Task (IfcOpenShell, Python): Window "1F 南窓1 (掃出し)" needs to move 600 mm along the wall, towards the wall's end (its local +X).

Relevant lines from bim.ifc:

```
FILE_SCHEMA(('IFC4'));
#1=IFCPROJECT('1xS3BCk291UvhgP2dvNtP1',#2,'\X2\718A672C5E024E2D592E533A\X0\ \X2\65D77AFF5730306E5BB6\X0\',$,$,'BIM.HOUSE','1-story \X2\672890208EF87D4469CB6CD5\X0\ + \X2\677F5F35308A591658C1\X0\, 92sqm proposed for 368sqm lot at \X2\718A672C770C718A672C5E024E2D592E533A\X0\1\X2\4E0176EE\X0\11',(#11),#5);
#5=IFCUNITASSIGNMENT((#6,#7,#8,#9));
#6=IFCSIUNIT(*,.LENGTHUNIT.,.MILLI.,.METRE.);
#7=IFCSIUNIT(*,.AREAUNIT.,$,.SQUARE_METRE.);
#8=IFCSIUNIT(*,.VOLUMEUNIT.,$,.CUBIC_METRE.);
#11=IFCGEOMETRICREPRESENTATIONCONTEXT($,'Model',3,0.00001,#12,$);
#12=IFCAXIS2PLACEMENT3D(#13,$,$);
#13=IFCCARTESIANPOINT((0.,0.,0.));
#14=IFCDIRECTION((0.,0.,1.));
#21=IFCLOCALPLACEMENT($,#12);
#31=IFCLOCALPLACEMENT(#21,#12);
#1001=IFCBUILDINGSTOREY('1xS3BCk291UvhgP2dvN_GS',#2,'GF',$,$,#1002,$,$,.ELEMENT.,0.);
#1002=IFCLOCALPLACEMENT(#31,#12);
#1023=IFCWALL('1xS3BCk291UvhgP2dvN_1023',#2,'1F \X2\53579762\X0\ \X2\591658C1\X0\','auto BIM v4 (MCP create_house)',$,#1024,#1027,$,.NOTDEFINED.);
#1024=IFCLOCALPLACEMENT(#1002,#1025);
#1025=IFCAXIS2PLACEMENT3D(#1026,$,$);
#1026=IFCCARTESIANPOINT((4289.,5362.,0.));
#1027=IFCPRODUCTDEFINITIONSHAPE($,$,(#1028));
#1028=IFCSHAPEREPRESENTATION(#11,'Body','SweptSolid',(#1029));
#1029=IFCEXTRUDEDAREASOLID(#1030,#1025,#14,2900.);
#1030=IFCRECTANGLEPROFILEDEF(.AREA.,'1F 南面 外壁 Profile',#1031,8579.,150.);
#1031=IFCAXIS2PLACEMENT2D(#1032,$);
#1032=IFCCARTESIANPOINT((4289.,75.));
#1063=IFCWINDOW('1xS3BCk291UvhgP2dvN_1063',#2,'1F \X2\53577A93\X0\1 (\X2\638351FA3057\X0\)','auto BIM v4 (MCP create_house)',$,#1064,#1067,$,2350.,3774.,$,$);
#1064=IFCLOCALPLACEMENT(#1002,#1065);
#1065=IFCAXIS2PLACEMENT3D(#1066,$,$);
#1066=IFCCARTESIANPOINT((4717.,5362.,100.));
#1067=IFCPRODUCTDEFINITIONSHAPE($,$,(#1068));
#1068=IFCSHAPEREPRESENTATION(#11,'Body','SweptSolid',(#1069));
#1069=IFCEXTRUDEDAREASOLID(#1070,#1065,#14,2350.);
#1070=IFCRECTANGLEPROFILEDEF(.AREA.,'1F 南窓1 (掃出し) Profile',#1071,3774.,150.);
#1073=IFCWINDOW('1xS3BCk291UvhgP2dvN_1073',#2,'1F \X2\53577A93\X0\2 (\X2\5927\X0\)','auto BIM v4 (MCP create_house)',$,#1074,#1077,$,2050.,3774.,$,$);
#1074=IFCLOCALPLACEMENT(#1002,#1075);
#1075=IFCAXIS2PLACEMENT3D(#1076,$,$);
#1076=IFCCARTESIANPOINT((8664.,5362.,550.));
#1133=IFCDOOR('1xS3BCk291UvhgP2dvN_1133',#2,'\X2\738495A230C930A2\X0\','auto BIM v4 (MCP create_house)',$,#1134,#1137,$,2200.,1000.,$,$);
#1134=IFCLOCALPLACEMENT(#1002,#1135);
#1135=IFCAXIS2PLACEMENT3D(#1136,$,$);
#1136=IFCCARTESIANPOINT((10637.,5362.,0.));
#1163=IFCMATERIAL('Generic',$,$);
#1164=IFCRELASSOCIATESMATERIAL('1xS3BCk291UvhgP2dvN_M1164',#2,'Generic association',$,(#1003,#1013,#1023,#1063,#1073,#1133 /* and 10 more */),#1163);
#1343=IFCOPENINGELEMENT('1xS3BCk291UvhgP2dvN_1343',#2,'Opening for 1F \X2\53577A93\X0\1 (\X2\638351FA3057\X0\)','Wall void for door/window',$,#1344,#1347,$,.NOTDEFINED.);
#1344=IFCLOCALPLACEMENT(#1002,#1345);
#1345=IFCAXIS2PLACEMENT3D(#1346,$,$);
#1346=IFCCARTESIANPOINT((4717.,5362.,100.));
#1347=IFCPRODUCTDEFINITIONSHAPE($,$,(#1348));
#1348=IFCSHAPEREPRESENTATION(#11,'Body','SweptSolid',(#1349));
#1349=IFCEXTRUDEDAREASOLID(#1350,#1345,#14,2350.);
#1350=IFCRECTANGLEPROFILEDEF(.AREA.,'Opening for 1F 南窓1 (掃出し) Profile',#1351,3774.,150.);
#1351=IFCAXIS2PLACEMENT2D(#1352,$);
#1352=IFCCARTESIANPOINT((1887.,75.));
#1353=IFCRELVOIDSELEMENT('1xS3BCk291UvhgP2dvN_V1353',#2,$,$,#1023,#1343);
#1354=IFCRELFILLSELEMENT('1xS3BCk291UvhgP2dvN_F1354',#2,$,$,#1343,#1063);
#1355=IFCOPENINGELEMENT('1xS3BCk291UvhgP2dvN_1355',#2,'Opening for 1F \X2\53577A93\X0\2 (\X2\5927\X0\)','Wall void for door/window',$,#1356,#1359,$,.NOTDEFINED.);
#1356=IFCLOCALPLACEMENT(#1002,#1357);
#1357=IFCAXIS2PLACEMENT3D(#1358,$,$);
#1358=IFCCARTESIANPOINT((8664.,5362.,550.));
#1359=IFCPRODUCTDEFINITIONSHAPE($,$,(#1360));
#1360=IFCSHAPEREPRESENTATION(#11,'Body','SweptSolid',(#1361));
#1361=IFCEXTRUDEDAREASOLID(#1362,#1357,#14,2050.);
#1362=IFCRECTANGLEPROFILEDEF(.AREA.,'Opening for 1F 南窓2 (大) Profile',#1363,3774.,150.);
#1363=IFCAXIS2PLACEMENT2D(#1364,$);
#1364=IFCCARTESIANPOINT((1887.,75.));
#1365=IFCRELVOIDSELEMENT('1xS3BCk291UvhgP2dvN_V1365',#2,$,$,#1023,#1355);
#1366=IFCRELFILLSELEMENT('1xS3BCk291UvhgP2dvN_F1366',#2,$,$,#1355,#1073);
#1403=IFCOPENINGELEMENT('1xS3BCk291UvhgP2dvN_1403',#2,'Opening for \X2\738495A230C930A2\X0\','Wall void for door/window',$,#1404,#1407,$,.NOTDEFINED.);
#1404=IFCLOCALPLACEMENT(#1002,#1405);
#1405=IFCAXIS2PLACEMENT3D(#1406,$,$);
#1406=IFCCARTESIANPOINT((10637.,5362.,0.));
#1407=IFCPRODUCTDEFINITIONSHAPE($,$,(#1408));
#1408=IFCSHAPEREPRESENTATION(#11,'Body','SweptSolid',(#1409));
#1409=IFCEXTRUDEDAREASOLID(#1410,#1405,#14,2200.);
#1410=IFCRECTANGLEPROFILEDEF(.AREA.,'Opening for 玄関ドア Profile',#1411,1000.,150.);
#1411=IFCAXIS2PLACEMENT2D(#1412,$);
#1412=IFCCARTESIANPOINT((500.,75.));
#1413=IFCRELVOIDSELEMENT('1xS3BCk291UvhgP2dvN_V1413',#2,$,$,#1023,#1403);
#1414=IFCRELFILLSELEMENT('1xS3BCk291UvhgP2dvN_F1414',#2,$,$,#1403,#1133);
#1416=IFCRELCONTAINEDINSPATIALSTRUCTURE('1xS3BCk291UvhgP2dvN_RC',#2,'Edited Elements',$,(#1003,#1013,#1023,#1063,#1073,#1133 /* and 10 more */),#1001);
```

```python
import ifcopenshell
import ifcopenshell.api.geometry
import ifcopenshell.util.placement

model = ifcopenshell.open("bim.ifc")

window = model.by_id(1063)
opening = window.FillsVoids[0].RelatingOpeningElement
wall = opening.VoidsElements[0].RelatingBuildingElement

wall_matrix = ifcopenshell.util.placement.get_local_placement(wall.ObjectPlacement)
shift = wall_matrix[:3, 0] * 600.0
before = ifcopenshell.util.placement.get_local_placement(window.ObjectPlacement)[:3, 3].copy()

# The window is not placed relative to its opening, so move both.
for product in (opening, window):
    matrix = ifcopenshell.util.placement.get_local_placement(product.ObjectPlacement)
    matrix[:3, 3] += shift
    ifcopenshell.api.geometry.edit_object_placement(model, product=product, matrix=matrix, is_si=False)

after = ifcopenshell.util.placement.get_local_placement(window.ObjectPlacement)[:3, 3]
print("window moved by", (after - before).round(3) + 0.0)

model.write("bim-out.ifc")
```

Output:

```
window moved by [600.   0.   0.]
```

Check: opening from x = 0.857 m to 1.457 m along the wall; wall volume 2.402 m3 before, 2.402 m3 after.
